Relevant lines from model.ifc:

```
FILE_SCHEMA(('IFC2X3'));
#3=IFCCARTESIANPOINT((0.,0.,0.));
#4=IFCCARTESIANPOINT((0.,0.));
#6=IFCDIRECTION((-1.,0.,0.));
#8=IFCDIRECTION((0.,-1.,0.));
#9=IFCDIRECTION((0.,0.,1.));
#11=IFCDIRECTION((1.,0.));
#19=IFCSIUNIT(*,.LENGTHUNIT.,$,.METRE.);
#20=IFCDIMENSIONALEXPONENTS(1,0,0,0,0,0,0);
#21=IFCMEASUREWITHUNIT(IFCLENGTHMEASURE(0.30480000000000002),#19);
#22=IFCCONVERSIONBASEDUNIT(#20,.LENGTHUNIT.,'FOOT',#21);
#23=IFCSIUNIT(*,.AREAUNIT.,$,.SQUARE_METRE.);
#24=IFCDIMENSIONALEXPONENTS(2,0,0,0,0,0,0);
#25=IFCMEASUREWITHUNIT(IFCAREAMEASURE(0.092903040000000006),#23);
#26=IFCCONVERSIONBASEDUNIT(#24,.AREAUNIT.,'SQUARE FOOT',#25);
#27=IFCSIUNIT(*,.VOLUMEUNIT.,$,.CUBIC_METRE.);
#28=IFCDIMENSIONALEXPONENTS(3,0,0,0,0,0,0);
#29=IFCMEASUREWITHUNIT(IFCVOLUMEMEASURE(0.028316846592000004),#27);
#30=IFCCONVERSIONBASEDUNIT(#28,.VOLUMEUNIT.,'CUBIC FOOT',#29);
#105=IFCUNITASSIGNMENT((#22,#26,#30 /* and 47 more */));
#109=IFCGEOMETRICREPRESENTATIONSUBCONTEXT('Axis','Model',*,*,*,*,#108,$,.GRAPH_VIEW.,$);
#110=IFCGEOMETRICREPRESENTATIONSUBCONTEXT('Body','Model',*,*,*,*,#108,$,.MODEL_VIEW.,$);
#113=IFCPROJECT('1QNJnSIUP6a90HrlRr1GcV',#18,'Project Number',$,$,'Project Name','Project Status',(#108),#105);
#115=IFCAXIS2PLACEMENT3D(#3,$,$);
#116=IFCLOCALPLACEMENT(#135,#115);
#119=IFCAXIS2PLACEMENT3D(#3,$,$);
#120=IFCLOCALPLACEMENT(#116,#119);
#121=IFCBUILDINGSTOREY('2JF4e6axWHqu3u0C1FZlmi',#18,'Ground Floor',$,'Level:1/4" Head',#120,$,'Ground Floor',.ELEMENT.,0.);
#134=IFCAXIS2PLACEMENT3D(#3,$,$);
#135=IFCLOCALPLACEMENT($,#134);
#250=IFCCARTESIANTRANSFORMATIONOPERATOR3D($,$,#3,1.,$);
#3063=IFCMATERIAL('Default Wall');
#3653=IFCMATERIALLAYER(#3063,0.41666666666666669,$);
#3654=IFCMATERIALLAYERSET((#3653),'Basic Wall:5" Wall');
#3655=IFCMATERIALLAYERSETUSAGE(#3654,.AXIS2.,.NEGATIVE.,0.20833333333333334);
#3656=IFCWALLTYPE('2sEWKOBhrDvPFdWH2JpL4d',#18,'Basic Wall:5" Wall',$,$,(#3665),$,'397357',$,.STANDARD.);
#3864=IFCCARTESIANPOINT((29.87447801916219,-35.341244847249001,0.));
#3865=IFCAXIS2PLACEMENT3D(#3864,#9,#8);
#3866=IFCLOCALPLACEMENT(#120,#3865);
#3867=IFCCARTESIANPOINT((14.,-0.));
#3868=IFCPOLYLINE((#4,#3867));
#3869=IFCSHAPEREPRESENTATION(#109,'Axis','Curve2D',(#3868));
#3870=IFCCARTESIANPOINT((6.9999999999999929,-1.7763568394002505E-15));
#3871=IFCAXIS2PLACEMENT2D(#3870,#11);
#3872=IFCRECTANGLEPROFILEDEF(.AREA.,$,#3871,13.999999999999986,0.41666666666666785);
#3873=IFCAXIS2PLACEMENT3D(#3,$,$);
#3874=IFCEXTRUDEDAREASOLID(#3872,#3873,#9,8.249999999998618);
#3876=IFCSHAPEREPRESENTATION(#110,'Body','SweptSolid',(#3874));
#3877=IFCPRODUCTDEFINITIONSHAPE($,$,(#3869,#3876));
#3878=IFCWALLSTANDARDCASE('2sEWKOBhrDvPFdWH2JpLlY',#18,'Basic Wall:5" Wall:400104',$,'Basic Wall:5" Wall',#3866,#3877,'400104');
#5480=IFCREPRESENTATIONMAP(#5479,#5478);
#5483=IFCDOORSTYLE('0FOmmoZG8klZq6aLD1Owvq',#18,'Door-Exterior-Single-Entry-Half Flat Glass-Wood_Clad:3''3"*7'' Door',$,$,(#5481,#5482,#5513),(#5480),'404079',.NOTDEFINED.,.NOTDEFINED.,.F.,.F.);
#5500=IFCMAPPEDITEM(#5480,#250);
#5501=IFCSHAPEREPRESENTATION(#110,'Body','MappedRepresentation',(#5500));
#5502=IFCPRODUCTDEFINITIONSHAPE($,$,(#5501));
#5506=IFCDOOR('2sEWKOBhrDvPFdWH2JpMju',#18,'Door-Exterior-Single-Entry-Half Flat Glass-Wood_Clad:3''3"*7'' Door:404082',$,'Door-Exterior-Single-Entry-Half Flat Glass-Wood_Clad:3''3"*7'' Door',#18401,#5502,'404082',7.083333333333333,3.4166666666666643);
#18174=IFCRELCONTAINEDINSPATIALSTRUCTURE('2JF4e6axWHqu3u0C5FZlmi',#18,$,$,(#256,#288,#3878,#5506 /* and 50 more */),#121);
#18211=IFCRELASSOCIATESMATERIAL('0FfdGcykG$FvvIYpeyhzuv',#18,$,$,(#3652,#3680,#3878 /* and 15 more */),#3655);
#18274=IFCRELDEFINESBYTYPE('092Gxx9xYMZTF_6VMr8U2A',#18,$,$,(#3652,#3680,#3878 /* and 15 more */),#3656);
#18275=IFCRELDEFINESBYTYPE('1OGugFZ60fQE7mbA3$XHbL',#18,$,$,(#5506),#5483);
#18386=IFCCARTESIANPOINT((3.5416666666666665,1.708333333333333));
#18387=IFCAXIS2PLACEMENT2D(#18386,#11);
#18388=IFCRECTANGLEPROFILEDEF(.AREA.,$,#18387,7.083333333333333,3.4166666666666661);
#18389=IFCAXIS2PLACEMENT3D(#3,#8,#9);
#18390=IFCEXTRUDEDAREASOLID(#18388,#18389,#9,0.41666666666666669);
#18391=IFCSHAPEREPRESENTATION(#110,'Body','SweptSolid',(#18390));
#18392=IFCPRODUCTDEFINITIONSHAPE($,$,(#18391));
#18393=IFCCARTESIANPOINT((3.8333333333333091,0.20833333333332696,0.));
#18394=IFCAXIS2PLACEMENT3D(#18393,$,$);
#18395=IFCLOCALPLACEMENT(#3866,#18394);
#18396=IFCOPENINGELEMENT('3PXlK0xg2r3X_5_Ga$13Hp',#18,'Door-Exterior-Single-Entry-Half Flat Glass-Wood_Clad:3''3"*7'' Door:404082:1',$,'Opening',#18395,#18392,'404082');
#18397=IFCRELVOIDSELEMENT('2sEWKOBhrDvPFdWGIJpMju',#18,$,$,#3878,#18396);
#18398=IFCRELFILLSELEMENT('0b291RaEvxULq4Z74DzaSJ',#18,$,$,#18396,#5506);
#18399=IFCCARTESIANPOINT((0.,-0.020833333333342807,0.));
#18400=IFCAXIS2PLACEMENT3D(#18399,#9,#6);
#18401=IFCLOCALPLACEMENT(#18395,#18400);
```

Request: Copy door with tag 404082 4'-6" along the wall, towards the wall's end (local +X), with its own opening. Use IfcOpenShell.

```python
import ifcopenshell
import ifcopenshell.api.feature
import ifcopenshell.api.geometry
import ifcopenshell.api.root
import ifcopenshell.geom
import ifcopenshell.util.element
import ifcopenshell.util.placement
import ifcopenshell.util.shape
import ifcopenshell.util.unit

model = ifcopenshell.open("model.ifc")
unit_scale = ifcopenshell.util.unit.calculate_unit_scale(model)
settings = ifcopenshell.geom.settings()


def volume(element):
    """Net volume in cubic metres, openings subtracted."""
    shape = ifcopenshell.geom.create_shape(settings, element)
    return ifcopenshell.util.shape.get_volume(shape.geometry)


def reuse_history(source, copy):
    """copy_class also copies each property set's owner history, people and application; keep the originals."""
    for rel in copy.IsDefinedBy:
        if rel.is_a("IfcRelDefinesByProperties") and (history := rel.RelatingPropertyDefinition.OwnerHistory):
            rel.RelatingPropertyDefinition.OwnerHistory = source.OwnerHistory
            ifcopenshell.util.element.remove_deep2(model, history)


door = model.by_guid("2sEWKOBhrDvPFdWH2JpMju")
opening = door.FillsVoids[0].RelatingOpeningElement
wall = opening.VoidsElements[0].RelatingBuildingElement
before = volume(wall)
shift = ifcopenshell.util.placement.get_local_placement(wall.ObjectPlacement)[:3, 0] * 54 * 0.0254 / unit_scale

# copy_class copies the void relationship, type, container and properties, but no geometry.
new_opening = ifcopenshell.api.root.copy_class(model, product=opening)
new_opening.Representation = ifcopenshell.util.element.copy_deep(
    model, opening.Representation, exclude=["IfcGeometricRepresentationContext", "IfcRepresentationMap"]
)
new_opening.Name = 'Door-Exterior-Single-Entry-Half Flat Glass-Wood_Clad:3\'3"*7\' Door'
new_opening.Tag = None
new_door = ifcopenshell.api.root.copy_class(model, product=door)
new_door.Representation = ifcopenshell.util.element.copy_deep(
    model, door.Representation, exclude=["IfcGeometricRepresentationContext", "IfcRepresentationMap"]
)
new_door.Name = 'Door-Exterior-Single-Entry-Half Flat Glass-Wood_Clad:3\'3"*7\' Door'
new_door.Tag = None
reuse_history(door, new_door)
fills = ifcopenshell.api.feature.add_filling(model, opening=new_opening, element=new_door)
fills.OwnerHistory = new_door.OwnerHistory  # required in IFC2X3

for old, new in ((opening, new_opening), (door, new_door)):
    matrix = ifcopenshell.util.placement.get_local_placement(old.ObjectPlacement)
    matrix[:3, 3] += shift
    ifcopenshell.api.geometry.edit_object_placement(model, product=new, matrix=matrix, is_si=False)

after = volume(wall)

print(f"wall volume {before:.3f} -> {after:.3f} m3")

model.write("model_edited.ifc")
```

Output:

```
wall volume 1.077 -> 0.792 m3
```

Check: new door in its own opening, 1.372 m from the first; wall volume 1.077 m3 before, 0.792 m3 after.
